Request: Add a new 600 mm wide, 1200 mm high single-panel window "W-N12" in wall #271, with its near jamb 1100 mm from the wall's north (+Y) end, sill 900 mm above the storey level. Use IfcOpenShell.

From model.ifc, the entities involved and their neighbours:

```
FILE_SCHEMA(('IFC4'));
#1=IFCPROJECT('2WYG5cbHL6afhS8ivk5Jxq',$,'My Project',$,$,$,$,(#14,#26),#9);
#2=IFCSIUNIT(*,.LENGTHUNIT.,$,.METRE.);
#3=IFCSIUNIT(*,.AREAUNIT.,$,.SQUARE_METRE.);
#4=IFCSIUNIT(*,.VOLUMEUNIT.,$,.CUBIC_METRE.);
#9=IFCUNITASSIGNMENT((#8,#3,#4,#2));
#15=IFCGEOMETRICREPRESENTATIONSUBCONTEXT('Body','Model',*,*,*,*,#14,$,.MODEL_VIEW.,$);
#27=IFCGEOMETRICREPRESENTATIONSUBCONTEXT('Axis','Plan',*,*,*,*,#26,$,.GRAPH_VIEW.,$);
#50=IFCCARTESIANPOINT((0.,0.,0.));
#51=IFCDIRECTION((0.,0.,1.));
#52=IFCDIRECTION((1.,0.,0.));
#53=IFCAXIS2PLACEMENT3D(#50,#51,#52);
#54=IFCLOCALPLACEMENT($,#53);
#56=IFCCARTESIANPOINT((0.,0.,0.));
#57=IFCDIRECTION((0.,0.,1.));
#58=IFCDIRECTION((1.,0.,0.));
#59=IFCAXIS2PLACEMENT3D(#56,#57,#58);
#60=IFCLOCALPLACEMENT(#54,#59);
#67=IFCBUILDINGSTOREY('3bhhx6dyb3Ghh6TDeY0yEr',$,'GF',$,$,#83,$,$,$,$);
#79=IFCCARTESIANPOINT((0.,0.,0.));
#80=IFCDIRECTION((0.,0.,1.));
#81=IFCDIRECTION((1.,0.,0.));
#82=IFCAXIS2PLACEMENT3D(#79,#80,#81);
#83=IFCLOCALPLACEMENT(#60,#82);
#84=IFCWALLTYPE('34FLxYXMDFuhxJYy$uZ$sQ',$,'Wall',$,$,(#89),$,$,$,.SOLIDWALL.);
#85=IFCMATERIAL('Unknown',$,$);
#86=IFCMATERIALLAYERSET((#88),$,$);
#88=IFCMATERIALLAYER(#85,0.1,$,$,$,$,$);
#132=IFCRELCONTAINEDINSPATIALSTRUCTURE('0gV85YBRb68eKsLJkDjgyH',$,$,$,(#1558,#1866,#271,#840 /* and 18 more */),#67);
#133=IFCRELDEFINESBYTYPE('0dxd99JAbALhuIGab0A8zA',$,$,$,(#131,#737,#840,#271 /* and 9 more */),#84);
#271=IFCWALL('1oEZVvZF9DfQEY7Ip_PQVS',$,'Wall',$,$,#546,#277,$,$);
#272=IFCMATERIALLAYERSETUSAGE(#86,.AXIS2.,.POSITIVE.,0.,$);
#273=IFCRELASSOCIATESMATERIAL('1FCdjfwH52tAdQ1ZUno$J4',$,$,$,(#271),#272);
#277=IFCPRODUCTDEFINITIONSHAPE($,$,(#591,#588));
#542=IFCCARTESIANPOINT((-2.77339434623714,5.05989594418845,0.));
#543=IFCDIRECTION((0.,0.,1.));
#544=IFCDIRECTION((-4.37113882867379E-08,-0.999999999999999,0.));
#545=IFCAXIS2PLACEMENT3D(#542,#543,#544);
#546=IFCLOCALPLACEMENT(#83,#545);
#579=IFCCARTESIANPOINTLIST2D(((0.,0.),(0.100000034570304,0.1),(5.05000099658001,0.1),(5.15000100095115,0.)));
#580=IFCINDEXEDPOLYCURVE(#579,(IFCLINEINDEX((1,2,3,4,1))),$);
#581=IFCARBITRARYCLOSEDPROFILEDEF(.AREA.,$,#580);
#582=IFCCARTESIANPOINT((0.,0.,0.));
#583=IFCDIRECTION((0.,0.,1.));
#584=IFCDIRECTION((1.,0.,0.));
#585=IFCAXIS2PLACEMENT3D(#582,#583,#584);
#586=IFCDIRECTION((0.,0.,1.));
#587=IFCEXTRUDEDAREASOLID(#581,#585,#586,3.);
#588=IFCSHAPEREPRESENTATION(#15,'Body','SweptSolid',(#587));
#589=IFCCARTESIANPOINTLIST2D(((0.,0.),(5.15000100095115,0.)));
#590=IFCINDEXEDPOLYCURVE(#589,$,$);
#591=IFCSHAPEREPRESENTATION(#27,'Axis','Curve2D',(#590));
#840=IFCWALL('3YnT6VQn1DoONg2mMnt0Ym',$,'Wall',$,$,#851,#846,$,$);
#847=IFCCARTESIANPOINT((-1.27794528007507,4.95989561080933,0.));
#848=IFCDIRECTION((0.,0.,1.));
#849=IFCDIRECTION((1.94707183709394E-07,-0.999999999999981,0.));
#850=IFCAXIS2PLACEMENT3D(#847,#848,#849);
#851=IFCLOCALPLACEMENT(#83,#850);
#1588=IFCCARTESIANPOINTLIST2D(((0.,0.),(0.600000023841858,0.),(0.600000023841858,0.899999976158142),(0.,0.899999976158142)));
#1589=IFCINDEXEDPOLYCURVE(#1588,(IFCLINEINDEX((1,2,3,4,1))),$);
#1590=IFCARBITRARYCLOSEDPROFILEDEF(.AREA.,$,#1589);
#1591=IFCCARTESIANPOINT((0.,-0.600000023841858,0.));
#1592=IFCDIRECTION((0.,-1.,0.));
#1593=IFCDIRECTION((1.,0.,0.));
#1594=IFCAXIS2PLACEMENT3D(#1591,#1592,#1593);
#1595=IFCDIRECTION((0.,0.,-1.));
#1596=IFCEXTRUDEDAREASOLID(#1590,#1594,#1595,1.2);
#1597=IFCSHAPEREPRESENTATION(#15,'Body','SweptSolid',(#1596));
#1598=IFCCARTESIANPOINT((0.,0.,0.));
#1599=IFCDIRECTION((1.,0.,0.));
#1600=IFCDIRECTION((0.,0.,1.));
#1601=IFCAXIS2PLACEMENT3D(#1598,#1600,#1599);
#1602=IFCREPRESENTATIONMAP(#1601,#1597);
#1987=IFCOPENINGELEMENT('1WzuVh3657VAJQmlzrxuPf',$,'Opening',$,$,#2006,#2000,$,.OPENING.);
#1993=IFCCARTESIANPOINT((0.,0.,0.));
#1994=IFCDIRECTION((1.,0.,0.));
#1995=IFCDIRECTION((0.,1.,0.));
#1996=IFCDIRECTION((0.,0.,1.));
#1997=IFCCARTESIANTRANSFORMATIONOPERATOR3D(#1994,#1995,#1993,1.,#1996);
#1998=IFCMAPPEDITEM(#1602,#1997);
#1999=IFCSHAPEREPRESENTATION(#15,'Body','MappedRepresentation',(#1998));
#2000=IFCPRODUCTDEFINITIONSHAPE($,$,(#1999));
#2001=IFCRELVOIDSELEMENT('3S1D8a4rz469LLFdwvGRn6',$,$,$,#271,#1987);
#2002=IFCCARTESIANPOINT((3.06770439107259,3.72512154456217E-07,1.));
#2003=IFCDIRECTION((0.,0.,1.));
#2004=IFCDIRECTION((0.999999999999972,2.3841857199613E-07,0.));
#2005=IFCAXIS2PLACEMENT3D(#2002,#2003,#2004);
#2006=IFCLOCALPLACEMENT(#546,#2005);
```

```python
import numpy as np
import ifcopenshell
import ifcopenshell.api.feature
import ifcopenshell.api.geometry
import ifcopenshell.api.root
import ifcopenshell.api.spatial
import ifcopenshell.geom
import ifcopenshell.util.element
import ifcopenshell.util.placement
import ifcopenshell.util.representation
import ifcopenshell.util.shape
import ifcopenshell.util.unit

model = ifcopenshell.open("model.ifc")
unit_scale = ifcopenshell.util.unit.calculate_unit_scale(model)
settings = ifcopenshell.geom.settings()


def volume(element):
    """Net volume in cubic metres, openings subtracted."""
    shape = ifcopenshell.geom.create_shape(settings, element)
    return ifcopenshell.util.shape.get_volume(shape.geometry)


wall = model.by_id(271)
storey = ifcopenshell.util.element.get_container(wall, ifc_class="IfcBuildingStorey")
context = ifcopenshell.util.representation.get_context(model, "Model", "Body", "MODEL_VIEW")
before = volume(wall)

width, height, from_end, sill = 0.6, 1.2, 1.1, 0.9  # metres

# The wall runs along its own X axis, and the end named is its -X end.
wall_shape = ifcopenshell.geom.create_shape(settings, wall)
x, y, z = ifcopenshell.util.shape.get_vertices(wall_shape.geometry).T
start = x.min() + from_end
face, thickness = float(y.min()), float(y.max() - y.min())
wall_matrix = ifcopenshell.util.placement.get_local_placement(wall.ObjectPlacement)
level = ifcopenshell.util.placement.get_local_placement(storey.ObjectPlacement)[2, 3]


def in_wall(x, y):
    """Placement at x, y metres in the wall's axes, at sill height."""
    matrix = wall_matrix.copy()
    matrix[:, 3] = wall_matrix @ np.array([x / unit_scale, y / unit_scale, 0.0, 1.0])
    matrix[2, 3] = level + sill / unit_scale
    return matrix


# Opening: a box that overshoots both wall faces by 50 mm.
opening = ifcopenshell.api.root.create_entity(model, ifc_class="IfcOpeningElement", predefined_type="OPENING")
box = ifcopenshell.api.geometry.add_wall_representation(
    model, context=context, length=width, height=height, thickness=thickness + 0.1
)
ifcopenshell.api.geometry.assign_representation(model, product=opening, representation=box)
ifcopenshell.api.geometry.edit_object_placement(model, product=opening, matrix=in_wall(start, face - 0.05), is_si=False)
ifcopenshell.api.feature.add_feature(model, feature=opening, element=wall)

window = ifcopenshell.api.root.create_entity(model, ifc_class="IfcWindow", name="W-N12", predefined_type="WINDOW")
window.OverallWidth, window.OverallHeight = width / unit_scale, height / unit_scale
window.PartitioningType = "SINGLE_PANEL"
body = ifcopenshell.api.geometry.add_window_representation(
    model,
    context=context,
    overall_width=window.OverallWidth,
    overall_height=window.OverallHeight,
    partition_type="SINGLE_PANEL",
)
ifcopenshell.api.geometry.assign_representation(model, product=window, representation=body)
ifcopenshell.api.spatial.assign_container(model, products=[window], relating_structure=storey)
ifcopenshell.api.feature.add_filling(model, opening=opening, element=window)

# Centre the window in the wall's thickness.
ifcopenshell.api.geometry.edit_object_placement(model, product=window, matrix=in_wall(start, face), is_si=False)
window_shape = ifcopenshell.geom.create_shape(settings, window)
depth = ifcopenshell.util.shape.get_vertices(window_shape.geometry)[:, 1]
offset = face + thickness / 2 - (depth.min() + depth.max()) / 2
ifcopenshell.api.geometry.edit_object_placement(model, product=window, matrix=in_wall(start, offset), is_si=False)

after = volume(wall)

print(f"wall volume {before:.3f} -> {after:.3f} m3")

model.write("model_rev.ifc")
```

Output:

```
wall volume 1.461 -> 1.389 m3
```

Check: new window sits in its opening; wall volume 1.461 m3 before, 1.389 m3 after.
